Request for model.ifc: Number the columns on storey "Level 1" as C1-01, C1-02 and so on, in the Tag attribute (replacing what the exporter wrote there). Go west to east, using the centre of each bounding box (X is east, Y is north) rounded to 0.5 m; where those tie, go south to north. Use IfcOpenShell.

First a look at what the model holds.

```python
import ifcopenshell
import ifcopenshell.util.element
import ifcopenshell.util.placement

model = ifcopenshell.open("model.ifc")
print(model.schema)
storey = next(s for s in model.by_type("IfcBuildingStorey") if s.Name == "Level 1")
columns = [e for e in ifcopenshell.util.element.get_decomposition(storey) if e.is_a("IfcColumn")]
for e in sorted(columns, key=lambda e: e.id()):
    origin = ifcopenshell.util.placement.get_local_placement(e.ObjectPlacement)[:3, 3]
    print(e.id(), e.Tag, e.Name, origin.round(2) + 0.0, sep=" | ")
```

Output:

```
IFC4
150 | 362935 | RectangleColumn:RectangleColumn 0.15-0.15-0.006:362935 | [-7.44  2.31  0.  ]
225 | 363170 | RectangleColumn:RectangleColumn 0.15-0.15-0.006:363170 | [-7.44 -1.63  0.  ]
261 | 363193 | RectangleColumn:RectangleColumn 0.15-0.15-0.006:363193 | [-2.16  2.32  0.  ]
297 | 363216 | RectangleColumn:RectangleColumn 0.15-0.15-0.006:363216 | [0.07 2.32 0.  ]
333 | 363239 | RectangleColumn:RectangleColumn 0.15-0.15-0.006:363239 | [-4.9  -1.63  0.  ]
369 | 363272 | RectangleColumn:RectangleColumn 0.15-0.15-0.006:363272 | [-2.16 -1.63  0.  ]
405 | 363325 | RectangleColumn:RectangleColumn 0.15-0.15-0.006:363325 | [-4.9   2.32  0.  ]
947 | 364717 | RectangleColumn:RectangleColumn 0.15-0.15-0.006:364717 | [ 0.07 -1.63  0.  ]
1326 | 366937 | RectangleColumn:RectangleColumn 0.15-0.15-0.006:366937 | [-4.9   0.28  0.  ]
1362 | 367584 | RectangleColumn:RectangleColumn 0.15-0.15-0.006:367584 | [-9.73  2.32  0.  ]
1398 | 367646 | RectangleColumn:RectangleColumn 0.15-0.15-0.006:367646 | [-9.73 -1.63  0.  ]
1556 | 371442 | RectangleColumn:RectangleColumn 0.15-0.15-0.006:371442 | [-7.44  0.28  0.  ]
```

```python
import ifcopenshell
import ifcopenshell.geom
import ifcopenshell.util.element
import ifcopenshell.util.shape

model = ifcopenshell.open("model.ifc")
settings = ifcopenshell.geom.settings()
settings.set("use-world-coords", True)


def centre(element):
    shape = ifcopenshell.geom.create_shape(settings, element)
    return ifcopenshell.util.shape.get_bbox_centroid(shape.geometry)


storey = next(s for s in model.by_type("IfcBuildingStorey") if s.Name == "Level 1")
columns = [e for e in ifcopenshell.util.element.get_decomposition(storey) if e.is_a("IfcColumn")]

# Insertion points can sit at a corner or the storey origin, so sort by the geometry (in metres).
centres = {e: centre(e) for e in columns}
columns.sort(key=lambda e: (round(centres[e][0] / 0.5), centres[e][1]))

for i, e in enumerate(columns, start=1):
    number = f"C1-{i:02d}"
    e.Tag = number
    print(e.id(), number)

model.write("model-out.ifc")
```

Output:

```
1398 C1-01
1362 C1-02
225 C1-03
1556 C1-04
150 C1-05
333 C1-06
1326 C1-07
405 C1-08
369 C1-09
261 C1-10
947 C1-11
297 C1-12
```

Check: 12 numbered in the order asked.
